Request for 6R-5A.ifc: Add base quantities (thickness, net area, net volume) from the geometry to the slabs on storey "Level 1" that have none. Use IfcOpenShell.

First a look at what the model holds.

```python
import ifcopenshell
import ifcopenshell.util.element
import ifcopenshell.util.unit

model = ifcopenshell.open("6R-5A.ifc")
print(model.schema)
for unit_type in ("LENGTHUNIT", "AREAUNIT", "VOLUMEUNIT"):
    print(unit_type, ifcopenshell.util.unit.calculate_unit_scale(model, unit_type))
storey = next(s for s in model.by_type("IfcBuildingStorey") if s.Name == "Level 1")
slabs = [e for e in ifcopenshell.util.element.get_decomposition(storey) if e.is_a("IfcSlab")]
for e in sorted(slabs, key=lambda e: e.id()):
    print(e.id(), e.is_a(), e.Name, list(ifcopenshell.util.element.get_psets(e, qtos_only=True)), sep=" | ")
```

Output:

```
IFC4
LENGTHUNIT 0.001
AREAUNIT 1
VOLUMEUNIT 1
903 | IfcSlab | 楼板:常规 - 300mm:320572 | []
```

```python
import ifcopenshell
import ifcopenshell.api.pset
import ifcopenshell.geom
import ifcopenshell.util.element
import ifcopenshell.util.shape
import ifcopenshell.util.unit

model = ifcopenshell.open("6R-5A.ifc")
unit_scale = ifcopenshell.util.unit.calculate_unit_scale(model)
area_scale = ifcopenshell.util.unit.calculate_unit_scale(model, "AREAUNIT")
volume_scale = ifcopenshell.util.unit.calculate_unit_scale(model, "VOLUMEUNIT")
settings = ifcopenshell.geom.settings()

storey = next(s for s in model.by_type("IfcBuildingStorey") if s.Name == "Level 1")
slabs = [e for e in ifcopenshell.util.element.get_decomposition(storey) if e.is_a("IfcSlab")]

for e in sorted(slabs, key=lambda e: e.id()):
    if ifcopenshell.util.element.get_psets(e, qtos_only=True, should_inherit=False):
        continue
    # Geometry comes back in metres, in the element's own axes.
    shape = ifcopenshell.geom.create_shape(settings, e)
    values = {
        "Width": ifcopenshell.util.shape.get_z(shape.geometry) / unit_scale,
        "NetArea": ifcopenshell.util.shape.get_footprint_area(shape.geometry) / area_scale,
        "NetVolume": ifcopenshell.util.shape.get_volume(shape.geometry) / volume_scale,
    }
    qto = ifcopenshell.api.pset.add_qto(model, product=e, name="Qto_SlabBaseQuantities")
    ifcopenshell.api.pset.edit_qto(model, qto=qto, properties=values)
    print(e.id(), {k: round(v, 3) for k, v in values.items()})

model.write("6R-5A_updated.ifc")
```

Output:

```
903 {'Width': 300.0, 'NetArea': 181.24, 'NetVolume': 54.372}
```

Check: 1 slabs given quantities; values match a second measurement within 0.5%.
